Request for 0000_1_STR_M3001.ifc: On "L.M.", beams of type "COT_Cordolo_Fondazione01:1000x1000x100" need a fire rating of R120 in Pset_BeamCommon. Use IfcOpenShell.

First a look at what the model holds.

```python
import ifcopenshell
import ifcopenshell.util.element

model = ifcopenshell.open("0000_1_STR_M3001.ifc")
print(model.schema)
storey = next(s for s in model.by_type("IfcBuildingStorey") if s.Name == "L.M.")
beams = [e for e in ifcopenshell.util.element.get_decomposition(storey) if e.is_a("IfcBeam")]
seen = {}
for e in beams:
    element_type = ifcopenshell.util.element.get_type(e)
    key = (element_type.Name if element_type != e and element_type else None, ifcopenshell.util.element.get_pset(e, "Pset_BeamCommon", "FireRating"))
    seen[key] = seen.get(key, 0) + 1
for (name, value), count in sorted(seen.items(), key=str):
    print(count, "x", name, "|", value)
```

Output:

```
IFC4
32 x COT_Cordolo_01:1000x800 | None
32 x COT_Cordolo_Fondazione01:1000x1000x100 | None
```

```python
import ifcopenshell
import ifcopenshell.api.pset
import ifcopenshell.util.element

model = ifcopenshell.open("0000_1_STR_M3001.ifc")

storey = next(s for s in model.by_type("IfcBuildingStorey") if s.Name == "L.M.")
beams = [e for e in ifcopenshell.util.element.get_decomposition(storey) if e.is_a("IfcBeam")]

count = 0
for e in beams:
    element_type = ifcopenshell.util.element.get_type(e)
    if element_type in (None, e) or element_type.Name != "COT_Cordolo_Fondazione01:1000x1000x100":
        continue
    # add_pset returns the element's existing set when there is one.
    pset = ifcopenshell.api.pset.add_pset(model, product=e, name="Pset_BeamCommon")
    ifcopenshell.api.pset.edit_pset(model, pset=pset, properties={"FireRating": "R120"})
    count += 1

print(count, "beams updated")

model.write("0000_1_STR_M3001-out.ifc")
```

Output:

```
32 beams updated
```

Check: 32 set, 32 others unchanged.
